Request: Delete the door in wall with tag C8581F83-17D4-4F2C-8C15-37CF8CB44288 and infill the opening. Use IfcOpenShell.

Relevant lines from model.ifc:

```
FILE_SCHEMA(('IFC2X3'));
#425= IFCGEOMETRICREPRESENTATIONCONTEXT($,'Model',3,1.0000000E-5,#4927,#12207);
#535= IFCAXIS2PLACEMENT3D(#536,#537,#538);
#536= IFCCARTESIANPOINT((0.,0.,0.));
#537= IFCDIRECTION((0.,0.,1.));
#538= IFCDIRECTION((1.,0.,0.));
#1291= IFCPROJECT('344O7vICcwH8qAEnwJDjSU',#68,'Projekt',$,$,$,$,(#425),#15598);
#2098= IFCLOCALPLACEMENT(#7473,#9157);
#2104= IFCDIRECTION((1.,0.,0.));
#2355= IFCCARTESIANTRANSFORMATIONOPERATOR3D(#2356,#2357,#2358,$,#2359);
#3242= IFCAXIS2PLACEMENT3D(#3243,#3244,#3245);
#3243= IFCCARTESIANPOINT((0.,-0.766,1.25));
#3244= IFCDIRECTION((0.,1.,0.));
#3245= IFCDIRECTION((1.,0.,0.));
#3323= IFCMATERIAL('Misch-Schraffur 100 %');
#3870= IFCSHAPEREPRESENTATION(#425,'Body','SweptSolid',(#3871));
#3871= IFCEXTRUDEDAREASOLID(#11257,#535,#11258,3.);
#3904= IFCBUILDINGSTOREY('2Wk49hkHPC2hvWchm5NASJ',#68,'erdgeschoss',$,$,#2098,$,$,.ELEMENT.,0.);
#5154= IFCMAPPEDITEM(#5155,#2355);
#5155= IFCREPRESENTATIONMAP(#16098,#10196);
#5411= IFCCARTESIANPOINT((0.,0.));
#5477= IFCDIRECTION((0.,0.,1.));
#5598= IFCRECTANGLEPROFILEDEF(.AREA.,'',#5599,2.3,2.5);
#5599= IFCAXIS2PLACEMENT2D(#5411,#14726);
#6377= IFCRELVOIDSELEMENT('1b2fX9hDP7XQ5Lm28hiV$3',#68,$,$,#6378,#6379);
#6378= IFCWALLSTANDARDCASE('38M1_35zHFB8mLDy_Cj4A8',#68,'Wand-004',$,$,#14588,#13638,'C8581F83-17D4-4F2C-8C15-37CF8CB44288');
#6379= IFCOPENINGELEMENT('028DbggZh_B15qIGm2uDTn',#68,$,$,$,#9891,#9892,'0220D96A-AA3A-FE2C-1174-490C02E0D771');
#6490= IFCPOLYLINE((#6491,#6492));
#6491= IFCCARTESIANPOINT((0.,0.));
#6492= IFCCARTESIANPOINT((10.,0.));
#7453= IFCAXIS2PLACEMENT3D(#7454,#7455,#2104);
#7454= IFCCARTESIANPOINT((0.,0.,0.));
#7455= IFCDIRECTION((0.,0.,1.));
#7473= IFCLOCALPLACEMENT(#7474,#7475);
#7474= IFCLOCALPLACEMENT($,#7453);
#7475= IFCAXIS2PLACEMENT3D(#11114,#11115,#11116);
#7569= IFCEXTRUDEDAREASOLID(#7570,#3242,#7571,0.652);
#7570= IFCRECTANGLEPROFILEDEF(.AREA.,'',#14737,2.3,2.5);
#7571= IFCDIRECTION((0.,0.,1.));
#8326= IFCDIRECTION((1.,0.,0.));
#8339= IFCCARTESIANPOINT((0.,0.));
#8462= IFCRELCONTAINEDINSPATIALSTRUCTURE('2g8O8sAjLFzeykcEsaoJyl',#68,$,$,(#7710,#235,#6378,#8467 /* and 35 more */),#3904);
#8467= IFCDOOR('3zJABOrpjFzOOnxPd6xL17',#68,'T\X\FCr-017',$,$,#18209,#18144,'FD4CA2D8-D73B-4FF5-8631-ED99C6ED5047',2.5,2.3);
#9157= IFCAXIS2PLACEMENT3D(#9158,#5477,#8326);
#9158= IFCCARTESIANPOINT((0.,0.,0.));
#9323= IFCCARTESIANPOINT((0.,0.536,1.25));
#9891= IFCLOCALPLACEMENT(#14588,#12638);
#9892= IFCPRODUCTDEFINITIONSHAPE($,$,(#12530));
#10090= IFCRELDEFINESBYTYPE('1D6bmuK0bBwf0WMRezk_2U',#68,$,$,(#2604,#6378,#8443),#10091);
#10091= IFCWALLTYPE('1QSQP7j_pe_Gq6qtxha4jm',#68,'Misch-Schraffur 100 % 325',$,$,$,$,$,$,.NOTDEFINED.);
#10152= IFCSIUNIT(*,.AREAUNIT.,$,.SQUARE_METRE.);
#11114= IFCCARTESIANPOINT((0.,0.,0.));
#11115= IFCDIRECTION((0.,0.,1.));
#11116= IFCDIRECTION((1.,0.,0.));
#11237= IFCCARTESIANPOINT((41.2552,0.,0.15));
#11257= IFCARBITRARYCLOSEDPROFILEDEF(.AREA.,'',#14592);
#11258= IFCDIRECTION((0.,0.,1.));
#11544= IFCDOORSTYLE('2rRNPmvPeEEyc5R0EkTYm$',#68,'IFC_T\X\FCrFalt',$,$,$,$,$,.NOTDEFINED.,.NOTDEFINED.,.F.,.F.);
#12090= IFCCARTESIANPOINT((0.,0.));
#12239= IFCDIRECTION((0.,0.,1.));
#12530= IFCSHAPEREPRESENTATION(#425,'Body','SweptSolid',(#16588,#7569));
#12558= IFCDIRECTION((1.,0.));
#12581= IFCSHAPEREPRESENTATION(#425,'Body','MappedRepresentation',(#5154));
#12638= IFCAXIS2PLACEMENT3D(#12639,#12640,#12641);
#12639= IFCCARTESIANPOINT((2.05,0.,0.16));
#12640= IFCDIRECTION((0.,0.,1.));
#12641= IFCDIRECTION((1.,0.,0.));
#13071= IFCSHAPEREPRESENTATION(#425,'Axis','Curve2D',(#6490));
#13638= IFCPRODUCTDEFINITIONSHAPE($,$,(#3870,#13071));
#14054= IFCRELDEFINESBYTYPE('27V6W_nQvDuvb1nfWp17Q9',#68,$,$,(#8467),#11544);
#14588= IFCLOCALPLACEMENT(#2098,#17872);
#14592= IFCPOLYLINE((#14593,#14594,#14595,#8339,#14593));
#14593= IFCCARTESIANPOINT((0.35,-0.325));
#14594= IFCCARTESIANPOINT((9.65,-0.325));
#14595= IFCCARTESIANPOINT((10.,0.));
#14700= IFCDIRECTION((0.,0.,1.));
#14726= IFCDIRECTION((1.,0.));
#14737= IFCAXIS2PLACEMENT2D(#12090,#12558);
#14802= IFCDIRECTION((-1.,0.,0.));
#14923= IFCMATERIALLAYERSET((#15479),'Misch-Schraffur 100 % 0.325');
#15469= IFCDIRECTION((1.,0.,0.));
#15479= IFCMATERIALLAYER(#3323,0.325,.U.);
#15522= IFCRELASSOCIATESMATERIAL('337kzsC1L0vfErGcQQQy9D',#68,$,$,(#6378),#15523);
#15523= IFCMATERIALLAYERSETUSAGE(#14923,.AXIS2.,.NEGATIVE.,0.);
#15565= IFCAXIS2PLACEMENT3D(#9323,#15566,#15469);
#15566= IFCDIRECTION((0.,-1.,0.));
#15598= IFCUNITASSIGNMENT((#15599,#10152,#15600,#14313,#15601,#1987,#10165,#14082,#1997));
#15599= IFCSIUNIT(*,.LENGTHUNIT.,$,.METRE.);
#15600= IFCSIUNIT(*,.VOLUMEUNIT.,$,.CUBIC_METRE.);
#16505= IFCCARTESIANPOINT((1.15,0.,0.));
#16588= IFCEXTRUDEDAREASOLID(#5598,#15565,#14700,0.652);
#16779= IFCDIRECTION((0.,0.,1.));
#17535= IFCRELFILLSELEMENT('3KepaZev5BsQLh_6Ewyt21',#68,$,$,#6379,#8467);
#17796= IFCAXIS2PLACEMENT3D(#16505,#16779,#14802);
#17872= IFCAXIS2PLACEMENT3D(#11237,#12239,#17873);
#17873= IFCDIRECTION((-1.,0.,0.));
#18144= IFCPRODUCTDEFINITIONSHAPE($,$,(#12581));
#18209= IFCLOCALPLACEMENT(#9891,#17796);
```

```python
import ifcopenshell
import ifcopenshell.api.feature
import ifcopenshell.api.root
import ifcopenshell.geom
import ifcopenshell.util.shape

model = ifcopenshell.open("model.ifc")
settings = ifcopenshell.geom.settings()


def volume(element):
    """Net volume in cubic metres, openings subtracted."""
    shape = ifcopenshell.geom.create_shape(settings, element)
    return ifcopenshell.util.shape.get_volume(shape.geometry)


door = model.by_guid("3zJABOrpjFzOOnxPd6xL17")
opening = door.FillsVoids[0].RelatingOpeningElement
wall = opening.VoidsElements[0].RelatingBuildingElement
before = volume(wall)

ifcopenshell.api.root.remove_product(model, product=door)
ifcopenshell.api.feature.remove_feature(model, feature=opening)

after = volume(wall)

print(f"wall volume {before:.3f} -> {after:.3f} m3")

model.write("model_edited.ifc")
```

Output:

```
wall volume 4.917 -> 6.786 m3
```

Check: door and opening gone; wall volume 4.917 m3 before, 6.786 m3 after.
